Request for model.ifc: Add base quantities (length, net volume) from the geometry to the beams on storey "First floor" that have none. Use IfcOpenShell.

First a look at what the model holds.

```python
import ifcopenshell
import ifcopenshell.util.element
import ifcopenshell.util.unit

model = ifcopenshell.open("model.ifc")
print(model.schema)
for unit_type in ("LENGTHUNIT", "AREAUNIT", "VOLUMEUNIT"):
    print(unit_type, ifcopenshell.util.unit.calculate_unit_scale(model, unit_type))
storey = next(s for s in model.by_type("IfcBuildingStorey") if s.Name == "First floor")
beams = [e for e in ifcopenshell.util.element.get_decomposition(storey) if e.is_a("IfcBeam")]
for e in sorted(beams, key=lambda e: e.id()):
    print(e.id(), e.is_a(), e.Name, list(ifcopenshell.util.element.get_psets(e, qtos_only=True)), sep=" | ")
```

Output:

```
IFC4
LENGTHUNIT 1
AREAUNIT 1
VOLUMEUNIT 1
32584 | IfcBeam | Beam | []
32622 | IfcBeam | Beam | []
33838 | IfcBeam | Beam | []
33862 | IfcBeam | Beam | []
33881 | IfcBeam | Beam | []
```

```python
import ifcopenshell
import ifcopenshell.api.pset
import ifcopenshell.geom
import ifcopenshell.util.element
import ifcopenshell.util.shape
import ifcopenshell.util.unit

model = ifcopenshell.open("model.ifc")
unit_scale = ifcopenshell.util.unit.calculate_unit_scale(model)
volume_scale = ifcopenshell.util.unit.calculate_unit_scale(model, "VOLUMEUNIT")
settings = ifcopenshell.geom.settings()

storey = next(s for s in model.by_type("IfcBuildingStorey") if s.Name == "First floor")
beams = [e for e in ifcopenshell.util.element.get_decomposition(storey) if e.is_a("IfcBeam")]

for e in sorted(beams, key=lambda e: e.id()):
    if ifcopenshell.util.element.get_psets(e, qtos_only=True, should_inherit=False):
        continue
    # Geometry comes back in metres, in the element's own axes.
    shape = ifcopenshell.geom.create_shape(settings, e)
    values = {
        "Length": ifcopenshell.util.shape.get_max_xyz(shape.geometry) / unit_scale,
        "NetVolume": ifcopenshell.util.shape.get_volume(shape.geometry) / volume_scale,
    }
    qto = ifcopenshell.api.pset.add_qto(model, product=e, name="Qto_BeamBaseQuantities")
    ifcopenshell.api.pset.edit_qto(model, qto=qto, properties=values)
    print(e.id(), {k: round(v, 3) for k, v in values.items()})

model.write("model-out.ifc")
```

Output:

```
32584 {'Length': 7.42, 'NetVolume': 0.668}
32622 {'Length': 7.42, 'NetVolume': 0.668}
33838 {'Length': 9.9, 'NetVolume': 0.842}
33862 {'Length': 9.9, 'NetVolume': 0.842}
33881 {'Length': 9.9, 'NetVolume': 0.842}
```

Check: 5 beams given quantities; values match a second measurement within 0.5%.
